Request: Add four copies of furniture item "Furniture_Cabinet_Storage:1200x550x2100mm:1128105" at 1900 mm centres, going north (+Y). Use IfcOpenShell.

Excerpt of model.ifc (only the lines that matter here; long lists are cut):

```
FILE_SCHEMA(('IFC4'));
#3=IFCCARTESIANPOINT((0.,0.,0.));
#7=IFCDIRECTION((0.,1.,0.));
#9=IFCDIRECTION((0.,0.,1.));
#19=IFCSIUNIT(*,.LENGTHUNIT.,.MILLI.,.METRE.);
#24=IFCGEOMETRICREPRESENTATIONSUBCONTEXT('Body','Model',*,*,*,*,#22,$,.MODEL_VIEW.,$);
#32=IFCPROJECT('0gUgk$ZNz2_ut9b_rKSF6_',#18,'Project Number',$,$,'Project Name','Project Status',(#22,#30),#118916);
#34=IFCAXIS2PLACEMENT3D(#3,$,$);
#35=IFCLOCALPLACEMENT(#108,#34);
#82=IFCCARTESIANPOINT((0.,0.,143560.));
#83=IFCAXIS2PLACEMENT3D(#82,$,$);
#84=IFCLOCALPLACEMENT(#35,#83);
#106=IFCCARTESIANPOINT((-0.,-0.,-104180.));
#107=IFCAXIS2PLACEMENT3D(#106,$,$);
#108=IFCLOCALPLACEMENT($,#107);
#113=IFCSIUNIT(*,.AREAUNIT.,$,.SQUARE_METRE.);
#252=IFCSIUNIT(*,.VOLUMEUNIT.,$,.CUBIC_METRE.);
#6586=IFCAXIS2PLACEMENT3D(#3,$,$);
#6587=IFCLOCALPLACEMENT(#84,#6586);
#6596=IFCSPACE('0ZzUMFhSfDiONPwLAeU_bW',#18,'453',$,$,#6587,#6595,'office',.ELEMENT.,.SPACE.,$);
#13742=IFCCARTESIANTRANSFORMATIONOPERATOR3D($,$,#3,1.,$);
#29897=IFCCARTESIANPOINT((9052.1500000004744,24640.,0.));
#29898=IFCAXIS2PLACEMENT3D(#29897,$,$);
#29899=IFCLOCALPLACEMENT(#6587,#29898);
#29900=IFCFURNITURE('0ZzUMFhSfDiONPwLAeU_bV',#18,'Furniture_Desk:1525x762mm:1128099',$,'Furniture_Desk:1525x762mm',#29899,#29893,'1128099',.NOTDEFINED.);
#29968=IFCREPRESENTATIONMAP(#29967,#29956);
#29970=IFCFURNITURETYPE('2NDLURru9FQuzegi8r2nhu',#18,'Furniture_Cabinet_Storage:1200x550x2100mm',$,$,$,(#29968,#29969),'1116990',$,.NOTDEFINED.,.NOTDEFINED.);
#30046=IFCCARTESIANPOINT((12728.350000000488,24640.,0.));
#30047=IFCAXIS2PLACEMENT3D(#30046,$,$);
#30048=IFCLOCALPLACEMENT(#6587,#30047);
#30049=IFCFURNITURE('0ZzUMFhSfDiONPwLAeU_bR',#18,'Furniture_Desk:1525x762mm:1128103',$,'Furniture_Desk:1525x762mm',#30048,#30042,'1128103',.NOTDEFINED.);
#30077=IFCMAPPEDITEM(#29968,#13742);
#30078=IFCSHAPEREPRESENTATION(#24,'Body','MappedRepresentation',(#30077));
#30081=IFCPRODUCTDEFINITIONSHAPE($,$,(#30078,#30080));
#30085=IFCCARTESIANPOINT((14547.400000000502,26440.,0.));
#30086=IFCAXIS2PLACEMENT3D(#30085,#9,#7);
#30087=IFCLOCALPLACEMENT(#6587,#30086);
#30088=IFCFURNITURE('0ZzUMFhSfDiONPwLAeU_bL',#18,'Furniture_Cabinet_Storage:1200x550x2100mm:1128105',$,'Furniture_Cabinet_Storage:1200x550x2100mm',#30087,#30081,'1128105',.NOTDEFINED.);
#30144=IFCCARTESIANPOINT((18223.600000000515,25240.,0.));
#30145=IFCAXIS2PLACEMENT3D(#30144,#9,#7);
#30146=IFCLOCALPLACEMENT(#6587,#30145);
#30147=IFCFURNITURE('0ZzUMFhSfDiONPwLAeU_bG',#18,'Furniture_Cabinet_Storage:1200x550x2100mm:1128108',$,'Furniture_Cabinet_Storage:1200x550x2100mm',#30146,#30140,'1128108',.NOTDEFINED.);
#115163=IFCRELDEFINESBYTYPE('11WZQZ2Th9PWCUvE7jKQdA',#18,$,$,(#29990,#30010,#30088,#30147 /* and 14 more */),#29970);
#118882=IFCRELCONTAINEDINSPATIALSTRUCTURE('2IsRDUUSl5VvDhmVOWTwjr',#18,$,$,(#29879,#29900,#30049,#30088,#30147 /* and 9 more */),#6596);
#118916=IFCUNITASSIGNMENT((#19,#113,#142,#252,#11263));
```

```python
import numpy as np
import ifcopenshell
import ifcopenshell.api.geometry
import ifcopenshell.api.root
import ifcopenshell.util.element
import ifcopenshell.util.placement

model = ifcopenshell.open("model.ifc")


def reuse_history(source, copy):
    """copy_class also copies each property set's owner history, people and application; keep the originals."""
    for rel in copy.IsDefinedBy:
        if rel.is_a("IfcRelDefinesByProperties") and (history := rel.RelatingPropertyDefinition.OwnerHistory):
            rel.RelatingPropertyDefinition.OwnerHistory = source.OwnerHistory
            ifcopenshell.util.element.remove_deep2(model, history)


source = model.by_guid("0ZzUMFhSfDiONPwLAeU_bL")
base = ifcopenshell.util.placement.get_local_placement(source.ObjectPlacement)
step = np.array([0.0, 1.0, 0.0]) * 1900.0

for i in range(1, 5):
    copy = ifcopenshell.api.root.copy_class(model, product=source)
    copy.Representation = ifcopenshell.util.element.copy_deep(
        model, source.Representation, exclude=["IfcGeometricRepresentationContext", "IfcRepresentationMap"]
    )
    copy.Name = "Furniture_Cabinet_Storage:1200x550x2100mm"
    copy.Tag = None
    reuse_history(source, copy)
    matrix = base.copy()
    matrix[:3, 3] += i * step
    print("added at", matrix[:3, 3].round(3) + 0.0)
    ifcopenshell.api.geometry.edit_object_placement(model, product=copy, matrix=matrix, is_si=False)

model.write("model_updated.ifc")
```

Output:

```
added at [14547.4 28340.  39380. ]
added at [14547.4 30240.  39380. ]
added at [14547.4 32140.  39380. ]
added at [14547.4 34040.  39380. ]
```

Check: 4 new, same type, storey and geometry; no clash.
